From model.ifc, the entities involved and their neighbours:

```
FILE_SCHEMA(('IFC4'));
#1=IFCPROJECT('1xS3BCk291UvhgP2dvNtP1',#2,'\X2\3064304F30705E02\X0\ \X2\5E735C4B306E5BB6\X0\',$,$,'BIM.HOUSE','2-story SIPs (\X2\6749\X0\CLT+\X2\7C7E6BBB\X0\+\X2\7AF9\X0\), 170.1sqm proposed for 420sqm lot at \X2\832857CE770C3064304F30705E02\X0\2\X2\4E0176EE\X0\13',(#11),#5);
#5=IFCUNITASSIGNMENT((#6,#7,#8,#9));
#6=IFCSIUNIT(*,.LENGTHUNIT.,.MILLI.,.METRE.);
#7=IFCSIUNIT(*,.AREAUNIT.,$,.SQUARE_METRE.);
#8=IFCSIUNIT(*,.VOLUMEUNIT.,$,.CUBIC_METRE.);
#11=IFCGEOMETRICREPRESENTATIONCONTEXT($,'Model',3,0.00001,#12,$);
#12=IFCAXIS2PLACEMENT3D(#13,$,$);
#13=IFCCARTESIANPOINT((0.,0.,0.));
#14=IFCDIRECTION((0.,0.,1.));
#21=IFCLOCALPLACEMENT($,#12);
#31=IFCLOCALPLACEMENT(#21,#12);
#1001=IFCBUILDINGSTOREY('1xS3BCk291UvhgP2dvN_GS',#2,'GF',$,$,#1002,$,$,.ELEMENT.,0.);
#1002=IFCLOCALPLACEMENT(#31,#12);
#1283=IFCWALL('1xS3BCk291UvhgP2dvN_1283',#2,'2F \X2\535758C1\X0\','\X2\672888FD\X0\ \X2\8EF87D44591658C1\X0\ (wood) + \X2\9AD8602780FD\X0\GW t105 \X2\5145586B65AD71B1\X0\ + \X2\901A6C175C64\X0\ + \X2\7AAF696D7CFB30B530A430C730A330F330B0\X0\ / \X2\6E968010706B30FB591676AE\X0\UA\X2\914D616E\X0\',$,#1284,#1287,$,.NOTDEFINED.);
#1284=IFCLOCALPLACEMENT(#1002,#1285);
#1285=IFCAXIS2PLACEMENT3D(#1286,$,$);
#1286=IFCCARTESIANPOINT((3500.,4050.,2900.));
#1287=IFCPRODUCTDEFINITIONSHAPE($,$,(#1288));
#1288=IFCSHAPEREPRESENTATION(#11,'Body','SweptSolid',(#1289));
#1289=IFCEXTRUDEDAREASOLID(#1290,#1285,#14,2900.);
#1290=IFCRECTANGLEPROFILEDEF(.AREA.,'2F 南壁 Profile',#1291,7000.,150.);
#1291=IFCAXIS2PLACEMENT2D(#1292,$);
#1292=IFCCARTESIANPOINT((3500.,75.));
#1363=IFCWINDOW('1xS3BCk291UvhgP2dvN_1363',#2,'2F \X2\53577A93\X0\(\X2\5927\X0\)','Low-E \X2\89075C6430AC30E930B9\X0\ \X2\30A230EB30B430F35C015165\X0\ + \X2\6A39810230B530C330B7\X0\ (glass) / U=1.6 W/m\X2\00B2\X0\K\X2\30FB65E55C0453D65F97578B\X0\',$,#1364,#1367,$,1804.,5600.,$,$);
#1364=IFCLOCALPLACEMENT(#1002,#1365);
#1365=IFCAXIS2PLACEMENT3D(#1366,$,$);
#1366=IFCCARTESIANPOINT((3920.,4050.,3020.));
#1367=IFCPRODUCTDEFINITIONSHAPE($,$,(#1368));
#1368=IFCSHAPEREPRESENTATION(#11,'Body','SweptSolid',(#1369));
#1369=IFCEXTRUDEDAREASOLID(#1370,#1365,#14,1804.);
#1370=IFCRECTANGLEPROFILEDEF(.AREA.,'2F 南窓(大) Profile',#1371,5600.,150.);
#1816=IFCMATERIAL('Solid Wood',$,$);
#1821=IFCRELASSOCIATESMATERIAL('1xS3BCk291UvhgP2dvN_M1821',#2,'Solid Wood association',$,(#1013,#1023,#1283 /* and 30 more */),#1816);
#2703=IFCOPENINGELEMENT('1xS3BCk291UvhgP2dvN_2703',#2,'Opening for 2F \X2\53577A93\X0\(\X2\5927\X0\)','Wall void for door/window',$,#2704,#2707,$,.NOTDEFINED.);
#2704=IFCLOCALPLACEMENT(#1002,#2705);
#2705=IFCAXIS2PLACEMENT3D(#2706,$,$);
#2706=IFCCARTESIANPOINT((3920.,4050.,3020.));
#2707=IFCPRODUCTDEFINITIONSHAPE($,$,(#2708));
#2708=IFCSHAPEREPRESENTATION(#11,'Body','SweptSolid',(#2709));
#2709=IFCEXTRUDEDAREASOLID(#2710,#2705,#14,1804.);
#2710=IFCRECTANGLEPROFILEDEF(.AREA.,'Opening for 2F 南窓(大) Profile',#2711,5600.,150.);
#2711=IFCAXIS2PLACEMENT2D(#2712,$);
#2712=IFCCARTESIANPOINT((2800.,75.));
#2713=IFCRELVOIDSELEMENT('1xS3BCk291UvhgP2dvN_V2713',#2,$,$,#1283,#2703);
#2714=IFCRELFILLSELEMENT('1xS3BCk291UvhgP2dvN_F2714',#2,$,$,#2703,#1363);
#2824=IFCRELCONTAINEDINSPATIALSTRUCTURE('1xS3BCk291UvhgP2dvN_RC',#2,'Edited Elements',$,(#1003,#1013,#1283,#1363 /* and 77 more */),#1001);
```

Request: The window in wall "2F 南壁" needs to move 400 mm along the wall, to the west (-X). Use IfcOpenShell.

```python
import ifcopenshell
import ifcopenshell.api.geometry
import ifcopenshell.util.placement

model = ifcopenshell.open("model.ifc")

window = model.by_guid("1xS3BCk291UvhgP2dvN_1363")
opening = window.FillsVoids[0].RelatingOpeningElement
wall = opening.VoidsElements[0].RelatingBuildingElement

wall_matrix = ifcopenshell.util.placement.get_local_placement(wall.ObjectPlacement)
shift = wall_matrix[:3, 0] * -400.0
before = ifcopenshell.util.placement.get_local_placement(window.ObjectPlacement)[:3, 3].copy()

# The window is not placed relative to its opening, so move both.
for product in (opening, window):
    matrix = ifcopenshell.util.placement.get_local_placement(product.ObjectPlacement)
    matrix[:3, 3] += shift
    ifcopenshell.api.geometry.edit_object_placement(model, product=product, matrix=matrix, is_si=False)

after = ifcopenshell.util.placement.get_local_placement(window.ObjectPlacement)[:3, 3]
print("window moved by", (after - before).round(3) + 0.0)

model.write("model-out.ifc")
```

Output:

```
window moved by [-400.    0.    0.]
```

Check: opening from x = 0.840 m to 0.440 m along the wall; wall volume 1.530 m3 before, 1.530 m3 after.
